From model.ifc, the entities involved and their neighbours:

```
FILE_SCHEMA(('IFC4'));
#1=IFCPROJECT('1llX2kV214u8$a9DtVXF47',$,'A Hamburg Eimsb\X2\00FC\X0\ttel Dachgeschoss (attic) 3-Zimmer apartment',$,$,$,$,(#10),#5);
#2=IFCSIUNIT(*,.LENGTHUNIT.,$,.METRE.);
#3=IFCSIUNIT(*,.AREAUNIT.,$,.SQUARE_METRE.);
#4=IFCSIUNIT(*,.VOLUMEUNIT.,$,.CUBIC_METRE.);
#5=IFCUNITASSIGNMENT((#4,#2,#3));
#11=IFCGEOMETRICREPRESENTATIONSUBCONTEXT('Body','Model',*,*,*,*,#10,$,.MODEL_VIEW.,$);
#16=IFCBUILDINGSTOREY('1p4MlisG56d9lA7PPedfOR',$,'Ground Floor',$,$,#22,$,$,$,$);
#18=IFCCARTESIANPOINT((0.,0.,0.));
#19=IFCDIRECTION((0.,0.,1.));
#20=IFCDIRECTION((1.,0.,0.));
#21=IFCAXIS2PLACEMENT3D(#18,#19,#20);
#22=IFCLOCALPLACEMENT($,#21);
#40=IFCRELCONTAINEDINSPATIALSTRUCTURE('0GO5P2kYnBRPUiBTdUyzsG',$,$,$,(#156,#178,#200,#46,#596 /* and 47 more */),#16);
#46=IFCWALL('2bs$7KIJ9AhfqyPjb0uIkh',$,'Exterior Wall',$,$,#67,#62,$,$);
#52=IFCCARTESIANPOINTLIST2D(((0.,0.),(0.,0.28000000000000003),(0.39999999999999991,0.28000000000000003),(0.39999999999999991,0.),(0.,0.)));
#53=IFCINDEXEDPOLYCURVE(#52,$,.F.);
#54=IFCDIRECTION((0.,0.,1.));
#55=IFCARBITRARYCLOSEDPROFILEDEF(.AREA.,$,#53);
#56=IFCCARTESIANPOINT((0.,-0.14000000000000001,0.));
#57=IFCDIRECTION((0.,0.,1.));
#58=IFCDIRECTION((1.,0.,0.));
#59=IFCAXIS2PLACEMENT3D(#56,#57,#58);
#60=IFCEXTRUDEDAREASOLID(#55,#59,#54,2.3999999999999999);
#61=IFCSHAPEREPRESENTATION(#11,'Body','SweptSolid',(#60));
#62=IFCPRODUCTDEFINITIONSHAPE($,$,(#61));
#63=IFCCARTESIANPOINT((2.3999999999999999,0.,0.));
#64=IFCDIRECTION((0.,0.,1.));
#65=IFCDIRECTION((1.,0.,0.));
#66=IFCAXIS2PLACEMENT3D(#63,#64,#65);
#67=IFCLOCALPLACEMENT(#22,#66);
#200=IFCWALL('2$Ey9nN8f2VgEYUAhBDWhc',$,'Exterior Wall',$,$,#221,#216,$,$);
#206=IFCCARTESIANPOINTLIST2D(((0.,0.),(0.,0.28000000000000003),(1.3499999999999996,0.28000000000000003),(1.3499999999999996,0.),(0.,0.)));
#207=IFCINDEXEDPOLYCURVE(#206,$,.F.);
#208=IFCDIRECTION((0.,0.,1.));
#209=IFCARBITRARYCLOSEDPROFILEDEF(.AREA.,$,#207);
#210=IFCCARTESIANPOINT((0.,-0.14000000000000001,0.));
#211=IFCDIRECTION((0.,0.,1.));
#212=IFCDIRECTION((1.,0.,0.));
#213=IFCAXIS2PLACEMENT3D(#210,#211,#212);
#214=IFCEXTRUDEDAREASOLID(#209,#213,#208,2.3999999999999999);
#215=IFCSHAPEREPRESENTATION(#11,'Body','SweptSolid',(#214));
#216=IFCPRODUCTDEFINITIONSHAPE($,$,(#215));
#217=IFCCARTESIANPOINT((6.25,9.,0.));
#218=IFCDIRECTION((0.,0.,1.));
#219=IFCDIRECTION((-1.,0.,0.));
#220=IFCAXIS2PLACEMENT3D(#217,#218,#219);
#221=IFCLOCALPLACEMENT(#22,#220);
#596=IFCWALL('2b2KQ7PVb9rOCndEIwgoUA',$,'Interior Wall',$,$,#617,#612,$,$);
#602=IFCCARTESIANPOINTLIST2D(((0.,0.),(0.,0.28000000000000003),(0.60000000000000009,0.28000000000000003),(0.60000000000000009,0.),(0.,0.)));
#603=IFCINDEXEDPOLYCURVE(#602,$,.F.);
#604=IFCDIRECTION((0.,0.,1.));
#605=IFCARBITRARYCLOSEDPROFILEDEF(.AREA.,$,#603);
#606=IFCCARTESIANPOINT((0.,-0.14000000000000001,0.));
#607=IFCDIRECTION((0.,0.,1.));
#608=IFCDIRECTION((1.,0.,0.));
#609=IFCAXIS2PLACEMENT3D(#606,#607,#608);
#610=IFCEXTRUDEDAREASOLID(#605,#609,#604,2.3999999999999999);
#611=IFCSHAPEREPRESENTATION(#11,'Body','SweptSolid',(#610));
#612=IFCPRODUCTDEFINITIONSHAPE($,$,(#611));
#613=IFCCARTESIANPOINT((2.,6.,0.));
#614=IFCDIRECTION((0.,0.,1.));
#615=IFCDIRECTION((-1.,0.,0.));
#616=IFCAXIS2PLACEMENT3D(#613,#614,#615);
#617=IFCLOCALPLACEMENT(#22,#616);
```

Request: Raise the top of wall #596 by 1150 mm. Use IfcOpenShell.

```python
import ifcopenshell
import ifcopenshell.geom
import ifcopenshell.util.representation
import ifcopenshell.util.shape
import ifcopenshell.util.unit

model = ifcopenshell.open("model.ifc")
unit_scale = ifcopenshell.util.unit.calculate_unit_scale(model)
settings = ifcopenshell.geom.settings()


def volume(element):
    """Net volume in cubic metres, openings subtracted."""
    shape = ifcopenshell.geom.create_shape(settings, element)
    return ifcopenshell.util.shape.get_volume(shape.geometry)


wall = model.by_guid("2b2KQ7PVb9rOCndEIwgoUA")
before = volume(wall)

body = ifcopenshell.util.representation.get_representation(wall, "Model", "Body")
solid = body.Items[0]
old_height = solid.Depth
solid.Depth += 1.15 / unit_scale
after = volume(wall)

print(f"height {old_height:g} -> {solid.Depth:g}, volume {before:.3f} -> {after:.3f} m3")

model.write("model_updated.ifc")
```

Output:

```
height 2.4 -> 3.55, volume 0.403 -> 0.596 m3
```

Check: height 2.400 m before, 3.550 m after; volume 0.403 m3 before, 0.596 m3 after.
